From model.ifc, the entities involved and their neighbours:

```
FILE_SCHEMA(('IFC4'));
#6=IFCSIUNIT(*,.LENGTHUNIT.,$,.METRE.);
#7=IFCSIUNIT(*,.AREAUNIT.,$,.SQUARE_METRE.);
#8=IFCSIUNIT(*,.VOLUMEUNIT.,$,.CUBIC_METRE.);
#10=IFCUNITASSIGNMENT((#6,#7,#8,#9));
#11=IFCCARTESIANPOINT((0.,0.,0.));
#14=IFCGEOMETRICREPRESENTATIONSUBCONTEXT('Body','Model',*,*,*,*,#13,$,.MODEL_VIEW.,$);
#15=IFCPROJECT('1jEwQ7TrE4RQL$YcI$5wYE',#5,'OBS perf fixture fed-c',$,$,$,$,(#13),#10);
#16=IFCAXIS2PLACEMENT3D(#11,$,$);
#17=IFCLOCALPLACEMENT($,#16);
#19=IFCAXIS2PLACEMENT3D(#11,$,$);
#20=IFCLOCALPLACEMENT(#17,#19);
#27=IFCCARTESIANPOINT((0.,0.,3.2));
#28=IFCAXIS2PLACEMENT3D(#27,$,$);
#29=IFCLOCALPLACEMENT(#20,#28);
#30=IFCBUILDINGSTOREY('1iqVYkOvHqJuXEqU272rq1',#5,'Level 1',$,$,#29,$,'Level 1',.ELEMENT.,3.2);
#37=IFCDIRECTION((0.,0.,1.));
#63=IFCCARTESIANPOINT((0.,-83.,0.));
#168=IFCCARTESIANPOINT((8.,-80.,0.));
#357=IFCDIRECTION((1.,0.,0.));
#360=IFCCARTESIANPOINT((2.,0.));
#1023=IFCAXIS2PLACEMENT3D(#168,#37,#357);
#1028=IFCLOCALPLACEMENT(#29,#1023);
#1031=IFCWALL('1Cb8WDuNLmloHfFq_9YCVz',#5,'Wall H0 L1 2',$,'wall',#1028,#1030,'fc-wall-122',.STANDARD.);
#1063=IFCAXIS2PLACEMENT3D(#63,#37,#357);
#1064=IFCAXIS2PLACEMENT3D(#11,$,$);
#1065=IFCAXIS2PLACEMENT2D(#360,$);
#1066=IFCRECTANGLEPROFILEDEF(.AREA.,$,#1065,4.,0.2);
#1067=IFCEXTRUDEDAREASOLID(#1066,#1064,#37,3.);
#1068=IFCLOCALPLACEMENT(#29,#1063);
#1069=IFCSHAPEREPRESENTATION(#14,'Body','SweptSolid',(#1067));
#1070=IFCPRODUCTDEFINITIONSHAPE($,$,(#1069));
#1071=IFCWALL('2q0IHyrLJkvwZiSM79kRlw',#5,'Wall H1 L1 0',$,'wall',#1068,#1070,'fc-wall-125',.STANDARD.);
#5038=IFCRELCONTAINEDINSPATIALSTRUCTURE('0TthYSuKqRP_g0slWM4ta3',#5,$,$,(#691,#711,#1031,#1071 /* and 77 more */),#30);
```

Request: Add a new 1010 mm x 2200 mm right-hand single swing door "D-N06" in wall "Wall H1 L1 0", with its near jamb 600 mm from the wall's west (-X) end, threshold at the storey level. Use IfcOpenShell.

```python
import numpy as np
import ifcopenshell
import ifcopenshell.api.feature
import ifcopenshell.api.geometry
import ifcopenshell.api.root
import ifcopenshell.api.spatial
import ifcopenshell.geom
import ifcopenshell.util.element
import ifcopenshell.util.placement
import ifcopenshell.util.representation
import ifcopenshell.util.shape
import ifcopenshell.util.unit

model = ifcopenshell.open("model.ifc")
unit_scale = ifcopenshell.util.unit.calculate_unit_scale(model)
settings = ifcopenshell.geom.settings()


def volume(element):
    """Net volume in cubic metres, openings subtracted."""
    shape = ifcopenshell.geom.create_shape(settings, element)
    return ifcopenshell.util.shape.get_volume(shape.geometry)


wall = model.by_guid("2q0IHyrLJkvwZiSM79kRlw")
storey = ifcopenshell.util.element.get_container(wall, ifc_class="IfcBuildingStorey")
context = ifcopenshell.util.representation.get_context(model, "Model", "Body", "MODEL_VIEW")
before = volume(wall)

width, height, from_end, sill = 1.01, 2.2, 0.6, 0.0  # metres

# The wall runs along its own X axis, and the end named is its -X end.
wall_shape = ifcopenshell.geom.create_shape(settings, wall)
x, y, z = ifcopenshell.util.shape.get_vertices(wall_shape.geometry).T
start = x.min() + from_end
face, thickness = float(y.min()), float(y.max() - y.min())
wall_matrix = ifcopenshell.util.placement.get_local_placement(wall.ObjectPlacement)
level = ifcopenshell.util.placement.get_local_placement(storey.ObjectPlacement)[2, 3]


def in_wall(x, y):
    """Placement at x, y metres in the wall's axes, at sill height."""
    matrix = wall_matrix.copy()
    matrix[:, 3] = wall_matrix @ np.array([x / unit_scale, y / unit_scale, 0.0, 1.0])
    matrix[2, 3] = level + sill / unit_scale
    return matrix


# Opening: a box that overshoots both wall faces by 50 mm.
opening = ifcopenshell.api.root.create_entity(model, ifc_class="IfcOpeningElement", predefined_type="OPENING")
box = ifcopenshell.api.geometry.add_wall_representation(
    model, context=context, length=width, height=height, thickness=thickness + 0.1
)
ifcopenshell.api.geometry.assign_representation(model, product=opening, representation=box)
ifcopenshell.api.geometry.edit_object_placement(model, product=opening, matrix=in_wall(start, face - 0.05), is_si=False)
ifcopenshell.api.feature.add_feature(model, feature=opening, element=wall)

door = ifcopenshell.api.root.create_entity(model, ifc_class="IfcDoor", name="D-N06", predefined_type="DOOR")
door.OverallWidth, door.OverallHeight = width / unit_scale, height / unit_scale
door.OperationType = "SINGLE_SWING_RIGHT"
body = ifcopenshell.api.geometry.add_door_representation(
    model,
    context=context,
    overall_width=door.OverallWidth,
    overall_height=door.OverallHeight,
    operation_type="SINGLE_SWING_RIGHT",
    lining_properties={"LiningDepth": thickness / unit_scale, "ThresholdDepth": thickness / unit_scale},
)
ifcopenshell.api.geometry.assign_representation(model, product=door, representation=body)
ifcopenshell.api.spatial.assign_container(model, products=[door], relating_structure=storey)
ifcopenshell.api.feature.add_filling(model, opening=opening, element=door)

# The lining spans the wall, so the door starts at the wall face.
ifcopenshell.api.geometry.edit_object_placement(model, product=door, matrix=in_wall(start, face), is_si=False)

after = volume(wall)

print(f"wall volume {before:.3f} -> {after:.3f} m3")

model.write("model-out.ifc")
```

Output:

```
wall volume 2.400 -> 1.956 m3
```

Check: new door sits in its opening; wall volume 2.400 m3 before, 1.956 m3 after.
